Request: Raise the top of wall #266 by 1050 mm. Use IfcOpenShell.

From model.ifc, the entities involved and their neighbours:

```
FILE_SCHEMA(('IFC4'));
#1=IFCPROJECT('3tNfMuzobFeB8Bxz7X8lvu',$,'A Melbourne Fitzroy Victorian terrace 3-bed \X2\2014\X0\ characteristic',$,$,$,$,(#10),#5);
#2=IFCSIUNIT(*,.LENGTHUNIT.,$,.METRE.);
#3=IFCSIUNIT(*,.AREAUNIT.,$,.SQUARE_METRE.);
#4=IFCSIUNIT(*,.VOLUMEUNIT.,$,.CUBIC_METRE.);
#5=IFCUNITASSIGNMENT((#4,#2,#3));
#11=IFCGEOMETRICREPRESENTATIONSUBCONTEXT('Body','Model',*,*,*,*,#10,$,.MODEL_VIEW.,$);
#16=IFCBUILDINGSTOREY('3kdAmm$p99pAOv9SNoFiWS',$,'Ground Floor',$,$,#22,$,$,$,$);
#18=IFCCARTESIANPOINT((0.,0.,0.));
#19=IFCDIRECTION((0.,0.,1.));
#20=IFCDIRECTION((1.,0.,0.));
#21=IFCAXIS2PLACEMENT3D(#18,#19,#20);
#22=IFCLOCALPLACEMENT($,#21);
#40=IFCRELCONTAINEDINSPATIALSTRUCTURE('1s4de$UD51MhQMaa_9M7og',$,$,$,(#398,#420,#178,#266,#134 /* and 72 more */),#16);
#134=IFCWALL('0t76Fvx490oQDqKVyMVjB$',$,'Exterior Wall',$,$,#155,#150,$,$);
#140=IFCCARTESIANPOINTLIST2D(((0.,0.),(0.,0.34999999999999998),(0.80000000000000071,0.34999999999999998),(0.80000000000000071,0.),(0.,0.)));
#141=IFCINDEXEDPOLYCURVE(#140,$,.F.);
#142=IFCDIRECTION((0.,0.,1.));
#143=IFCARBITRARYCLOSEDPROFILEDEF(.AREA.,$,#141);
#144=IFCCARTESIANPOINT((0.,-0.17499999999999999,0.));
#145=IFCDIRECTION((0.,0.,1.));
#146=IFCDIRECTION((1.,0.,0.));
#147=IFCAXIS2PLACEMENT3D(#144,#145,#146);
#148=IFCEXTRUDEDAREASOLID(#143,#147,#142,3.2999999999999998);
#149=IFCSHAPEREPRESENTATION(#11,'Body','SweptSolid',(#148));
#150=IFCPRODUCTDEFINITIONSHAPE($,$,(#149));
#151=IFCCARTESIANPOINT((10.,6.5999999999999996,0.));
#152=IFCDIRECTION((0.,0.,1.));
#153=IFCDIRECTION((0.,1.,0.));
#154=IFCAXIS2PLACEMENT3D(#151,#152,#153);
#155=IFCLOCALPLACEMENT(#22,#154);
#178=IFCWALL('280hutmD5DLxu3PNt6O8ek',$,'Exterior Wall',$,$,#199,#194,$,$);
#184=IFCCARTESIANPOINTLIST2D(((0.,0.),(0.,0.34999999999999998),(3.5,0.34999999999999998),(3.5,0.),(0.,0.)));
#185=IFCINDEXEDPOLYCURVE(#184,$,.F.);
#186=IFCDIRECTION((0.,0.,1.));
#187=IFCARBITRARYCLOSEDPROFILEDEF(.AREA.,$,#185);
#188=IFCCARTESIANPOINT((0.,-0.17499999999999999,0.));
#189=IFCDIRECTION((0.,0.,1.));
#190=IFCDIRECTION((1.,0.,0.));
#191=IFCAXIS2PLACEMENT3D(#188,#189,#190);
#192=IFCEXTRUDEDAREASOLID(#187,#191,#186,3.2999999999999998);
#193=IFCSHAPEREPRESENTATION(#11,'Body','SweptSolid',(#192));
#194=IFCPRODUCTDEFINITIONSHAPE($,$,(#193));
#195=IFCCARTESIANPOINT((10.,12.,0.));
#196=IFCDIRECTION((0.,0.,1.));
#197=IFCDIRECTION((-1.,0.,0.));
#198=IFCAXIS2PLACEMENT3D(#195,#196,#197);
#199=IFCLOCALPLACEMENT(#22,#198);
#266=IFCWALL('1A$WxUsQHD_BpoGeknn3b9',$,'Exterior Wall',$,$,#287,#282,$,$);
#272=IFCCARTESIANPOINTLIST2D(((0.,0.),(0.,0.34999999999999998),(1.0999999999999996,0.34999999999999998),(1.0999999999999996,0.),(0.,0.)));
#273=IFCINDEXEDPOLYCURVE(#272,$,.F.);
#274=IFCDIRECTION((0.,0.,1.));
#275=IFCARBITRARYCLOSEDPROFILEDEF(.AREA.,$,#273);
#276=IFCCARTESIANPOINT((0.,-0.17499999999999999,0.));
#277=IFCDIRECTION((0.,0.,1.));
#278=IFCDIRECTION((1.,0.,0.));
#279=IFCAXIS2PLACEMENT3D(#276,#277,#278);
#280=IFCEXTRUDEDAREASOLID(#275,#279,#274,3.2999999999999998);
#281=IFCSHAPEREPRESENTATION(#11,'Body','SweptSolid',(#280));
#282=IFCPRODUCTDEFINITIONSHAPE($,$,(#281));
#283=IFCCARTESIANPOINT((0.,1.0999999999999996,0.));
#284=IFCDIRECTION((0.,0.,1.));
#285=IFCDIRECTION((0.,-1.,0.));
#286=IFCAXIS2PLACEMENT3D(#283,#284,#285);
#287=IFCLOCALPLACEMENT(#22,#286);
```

```python
import ifcopenshell
import ifcopenshell.geom
import ifcopenshell.util.representation
import ifcopenshell.util.shape

model = ifcopenshell.open("model.ifc")
settings = ifcopenshell.geom.settings()


def volume(element):
    """Net volume in cubic metres, openings subtracted."""
    shape = ifcopenshell.geom.create_shape(settings, element)
    return ifcopenshell.util.shape.get_volume(shape.geometry)


wall = model.by_id(266)
before = volume(wall)

body = ifcopenshell.util.representation.get_representation(wall, "Model", "Body")
solid = body.Items[0]
old_height = solid.Depth
solid.Depth += 1.05
after = volume(wall)

print(f"height {old_height:g} -> {solid.Depth:g}, volume {before:.3f} -> {after:.3f} m3")

model.write("model_updated.ifc")
```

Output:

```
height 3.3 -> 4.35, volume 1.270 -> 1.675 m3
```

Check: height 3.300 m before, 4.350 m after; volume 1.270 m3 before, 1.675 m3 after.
